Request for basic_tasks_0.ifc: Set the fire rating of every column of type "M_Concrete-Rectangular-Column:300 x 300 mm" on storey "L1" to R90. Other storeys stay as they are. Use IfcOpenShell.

First a look at what the model holds.

```python
import ifcopenshell
import ifcopenshell.util.element

model = ifcopenshell.open("basic_tasks_0.ifc")
print(model.schema)
storey = next(s for s in model.by_type("IfcBuildingStorey") if s.Name == "L1")
columns = [e for e in ifcopenshell.util.element.get_decomposition(storey) if e.is_a("IfcColumn")]
seen = {}
for e in columns:
    element_type = ifcopenshell.util.element.get_type(e)
    key = (element_type.Name if element_type != e and element_type else None, ifcopenshell.util.element.get_pset(e, "Pset_ColumnCommon", "FireRating"))
    seen[key] = seen.get(key, 0) + 1
for (name, value), count in sorted(seen.items(), key=str):
    print(count, "x", name, "|", value)
```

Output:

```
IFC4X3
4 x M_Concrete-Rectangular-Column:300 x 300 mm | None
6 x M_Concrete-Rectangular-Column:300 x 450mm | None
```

```python
import ifcopenshell
import ifcopenshell.api.pset
import ifcopenshell.util.element

model = ifcopenshell.open("basic_tasks_0.ifc")

storey = next(s for s in model.by_type("IfcBuildingStorey") if s.Name == "L1")
columns = [e for e in ifcopenshell.util.element.get_decomposition(storey) if e.is_a("IfcColumn")]

count = 0
for e in columns:
    element_type = ifcopenshell.util.element.get_type(e)
    if element_type in (None, e) or element_type.Name != "M_Concrete-Rectangular-Column:300 x 300 mm":
        continue
    # add_pset returns the element's existing set when there is one.
    pset = ifcopenshell.api.pset.add_pset(model, product=e, name="Pset_ColumnCommon")
    ifcopenshell.api.pset.edit_pset(model, pset=pset, properties={"FireRating": "R90"})
    count += 1

print(count, "columns updated")

model.write("basic_tasks_0_edited.ifc")
```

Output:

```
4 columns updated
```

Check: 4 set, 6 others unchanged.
